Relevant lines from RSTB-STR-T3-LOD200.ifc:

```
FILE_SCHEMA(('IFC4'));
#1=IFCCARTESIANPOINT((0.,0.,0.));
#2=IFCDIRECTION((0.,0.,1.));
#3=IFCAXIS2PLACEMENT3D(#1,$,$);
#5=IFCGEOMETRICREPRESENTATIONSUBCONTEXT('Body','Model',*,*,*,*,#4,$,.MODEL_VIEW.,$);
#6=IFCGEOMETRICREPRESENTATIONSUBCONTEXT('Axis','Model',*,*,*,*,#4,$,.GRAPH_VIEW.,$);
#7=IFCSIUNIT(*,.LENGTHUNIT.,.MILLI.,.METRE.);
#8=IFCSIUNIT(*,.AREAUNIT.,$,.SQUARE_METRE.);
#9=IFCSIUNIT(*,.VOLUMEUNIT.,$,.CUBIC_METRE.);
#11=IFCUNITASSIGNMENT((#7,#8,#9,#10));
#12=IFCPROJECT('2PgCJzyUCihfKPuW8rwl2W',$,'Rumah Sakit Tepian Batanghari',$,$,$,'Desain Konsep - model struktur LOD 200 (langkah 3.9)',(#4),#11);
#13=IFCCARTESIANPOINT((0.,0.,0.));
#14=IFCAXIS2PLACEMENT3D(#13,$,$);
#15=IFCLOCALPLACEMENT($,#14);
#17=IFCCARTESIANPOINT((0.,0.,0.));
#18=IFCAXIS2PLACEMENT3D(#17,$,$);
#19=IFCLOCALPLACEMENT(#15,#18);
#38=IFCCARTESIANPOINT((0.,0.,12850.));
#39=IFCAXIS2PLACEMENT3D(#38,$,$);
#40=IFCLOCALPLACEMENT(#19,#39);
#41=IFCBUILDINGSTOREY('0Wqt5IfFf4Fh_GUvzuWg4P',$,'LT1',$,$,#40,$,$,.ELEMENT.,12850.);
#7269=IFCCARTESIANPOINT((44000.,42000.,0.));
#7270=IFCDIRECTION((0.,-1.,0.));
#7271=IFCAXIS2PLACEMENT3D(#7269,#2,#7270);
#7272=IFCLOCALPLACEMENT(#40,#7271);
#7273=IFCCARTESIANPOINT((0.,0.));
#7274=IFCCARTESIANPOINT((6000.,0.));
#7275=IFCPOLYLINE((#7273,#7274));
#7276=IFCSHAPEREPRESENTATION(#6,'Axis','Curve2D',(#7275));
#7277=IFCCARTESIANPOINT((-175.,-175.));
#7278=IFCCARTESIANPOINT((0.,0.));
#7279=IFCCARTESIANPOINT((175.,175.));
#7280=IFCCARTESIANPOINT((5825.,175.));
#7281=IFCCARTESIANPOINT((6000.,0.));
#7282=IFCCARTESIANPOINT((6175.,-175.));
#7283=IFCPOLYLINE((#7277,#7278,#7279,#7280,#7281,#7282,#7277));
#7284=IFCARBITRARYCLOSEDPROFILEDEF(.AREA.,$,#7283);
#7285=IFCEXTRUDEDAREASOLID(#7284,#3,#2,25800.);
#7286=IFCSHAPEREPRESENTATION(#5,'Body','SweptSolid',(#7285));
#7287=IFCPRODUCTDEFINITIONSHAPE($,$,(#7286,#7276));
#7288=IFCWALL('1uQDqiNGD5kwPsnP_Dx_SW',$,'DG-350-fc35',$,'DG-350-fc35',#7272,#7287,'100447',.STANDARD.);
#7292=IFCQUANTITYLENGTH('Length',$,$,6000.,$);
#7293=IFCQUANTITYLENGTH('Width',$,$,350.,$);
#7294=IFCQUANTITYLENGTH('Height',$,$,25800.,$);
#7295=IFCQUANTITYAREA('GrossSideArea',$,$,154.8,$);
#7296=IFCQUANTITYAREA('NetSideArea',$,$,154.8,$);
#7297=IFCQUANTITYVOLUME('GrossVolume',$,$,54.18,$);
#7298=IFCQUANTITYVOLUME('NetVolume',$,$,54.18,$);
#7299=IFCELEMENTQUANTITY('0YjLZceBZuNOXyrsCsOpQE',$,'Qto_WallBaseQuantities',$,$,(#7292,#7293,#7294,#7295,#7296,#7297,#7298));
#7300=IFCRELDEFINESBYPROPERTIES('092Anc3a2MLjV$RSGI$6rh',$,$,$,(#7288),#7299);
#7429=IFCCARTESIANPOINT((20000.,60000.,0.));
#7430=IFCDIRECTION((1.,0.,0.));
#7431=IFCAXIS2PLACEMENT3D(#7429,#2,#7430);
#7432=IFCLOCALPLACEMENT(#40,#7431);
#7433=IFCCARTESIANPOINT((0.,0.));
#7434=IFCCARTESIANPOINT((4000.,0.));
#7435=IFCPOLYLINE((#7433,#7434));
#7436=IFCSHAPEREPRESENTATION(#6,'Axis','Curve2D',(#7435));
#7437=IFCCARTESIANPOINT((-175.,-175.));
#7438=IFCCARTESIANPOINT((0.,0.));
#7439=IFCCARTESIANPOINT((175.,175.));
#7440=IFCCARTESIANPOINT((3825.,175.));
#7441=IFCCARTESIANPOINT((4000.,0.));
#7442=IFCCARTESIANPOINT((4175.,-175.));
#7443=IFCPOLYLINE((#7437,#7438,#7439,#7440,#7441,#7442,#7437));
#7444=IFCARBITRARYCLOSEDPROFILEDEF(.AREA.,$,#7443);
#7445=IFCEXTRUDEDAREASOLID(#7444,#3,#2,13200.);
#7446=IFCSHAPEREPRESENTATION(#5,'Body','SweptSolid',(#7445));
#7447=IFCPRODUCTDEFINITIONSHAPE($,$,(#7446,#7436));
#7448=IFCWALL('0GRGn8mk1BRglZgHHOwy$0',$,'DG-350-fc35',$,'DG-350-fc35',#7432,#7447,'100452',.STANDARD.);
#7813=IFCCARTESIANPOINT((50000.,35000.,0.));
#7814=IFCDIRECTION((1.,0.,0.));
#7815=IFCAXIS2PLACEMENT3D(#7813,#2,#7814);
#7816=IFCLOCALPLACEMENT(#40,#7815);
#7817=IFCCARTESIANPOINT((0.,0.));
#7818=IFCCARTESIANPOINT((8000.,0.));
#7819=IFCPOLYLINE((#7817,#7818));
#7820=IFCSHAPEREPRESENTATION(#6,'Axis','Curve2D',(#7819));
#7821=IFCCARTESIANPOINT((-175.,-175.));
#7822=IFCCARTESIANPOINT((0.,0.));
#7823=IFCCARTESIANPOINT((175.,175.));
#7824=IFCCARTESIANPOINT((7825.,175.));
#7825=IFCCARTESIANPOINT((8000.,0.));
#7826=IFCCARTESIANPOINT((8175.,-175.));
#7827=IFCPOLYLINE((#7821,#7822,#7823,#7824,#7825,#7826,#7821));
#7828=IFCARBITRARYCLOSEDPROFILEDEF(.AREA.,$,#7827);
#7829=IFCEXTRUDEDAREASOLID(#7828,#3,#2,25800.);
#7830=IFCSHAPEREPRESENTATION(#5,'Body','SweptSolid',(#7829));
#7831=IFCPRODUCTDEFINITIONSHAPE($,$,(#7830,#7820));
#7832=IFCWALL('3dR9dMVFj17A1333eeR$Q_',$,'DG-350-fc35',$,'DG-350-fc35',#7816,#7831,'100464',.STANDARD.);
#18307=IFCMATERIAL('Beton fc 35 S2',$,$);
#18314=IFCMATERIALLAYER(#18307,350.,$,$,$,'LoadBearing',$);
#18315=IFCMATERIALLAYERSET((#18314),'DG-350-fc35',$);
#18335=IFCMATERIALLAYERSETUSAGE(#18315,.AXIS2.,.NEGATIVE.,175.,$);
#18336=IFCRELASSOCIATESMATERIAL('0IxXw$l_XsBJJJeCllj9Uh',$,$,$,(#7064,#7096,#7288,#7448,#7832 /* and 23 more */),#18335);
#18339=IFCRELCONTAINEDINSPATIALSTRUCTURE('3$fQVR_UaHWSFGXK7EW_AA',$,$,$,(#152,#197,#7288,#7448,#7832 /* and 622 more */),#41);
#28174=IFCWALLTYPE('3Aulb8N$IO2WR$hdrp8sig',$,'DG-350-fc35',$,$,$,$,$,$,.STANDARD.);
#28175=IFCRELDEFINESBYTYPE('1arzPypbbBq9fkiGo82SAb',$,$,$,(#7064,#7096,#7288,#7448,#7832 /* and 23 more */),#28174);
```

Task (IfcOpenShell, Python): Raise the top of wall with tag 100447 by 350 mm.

```python
import ifcopenshell
import ifcopenshell.api.pset
import ifcopenshell.geom
import ifcopenshell.util.element
import ifcopenshell.util.representation
import ifcopenshell.util.shape
import ifcopenshell.util.unit

model = ifcopenshell.open("RSTB-STR-T3-LOD200.ifc")
unit_scale = ifcopenshell.util.unit.calculate_unit_scale(model)
area_scale = ifcopenshell.util.unit.calculate_unit_scale(model, "AREAUNIT")
volume_scale = ifcopenshell.util.unit.calculate_unit_scale(model, "VOLUMEUNIT")
settings = ifcopenshell.geom.settings()


def volume(element):
    """Net volume in cubic metres, openings subtracted."""
    shape = ifcopenshell.geom.create_shape(settings, element)
    return ifcopenshell.util.shape.get_volume(shape.geometry)


wall = model.by_guid("1uQDqiNGD5kwPsnP_Dx_SW")
before = volume(wall)

body = ifcopenshell.util.representation.get_representation(wall, "Model", "Body")
solid = body.Items[0]
old_height = solid.Depth
solid.Depth += 350.0
after = volume(wall)
thickness = 0.35  # wall thickness in metres

# Update the stored height, areas and volumes.
qto = model.by_id(ifcopenshell.util.element.get_pset(wall, "Qto_WallBaseQuantities", should_inherit=False)["id"])
ifcopenshell.api.pset.edit_qto(model, qto=qto, properties={
    "Height": solid.Depth,
    "GrossSideArea": ifcopenshell.util.element.get_pset(wall, "Qto_WallBaseQuantities", "GrossSideArea") * solid.Depth / old_height,
    "NetSideArea": after / thickness / area_scale,
    "GrossVolume": ifcopenshell.util.element.get_pset(wall, "Qto_WallBaseQuantities", "GrossVolume") * solid.Depth / old_height,
    "NetVolume": after / volume_scale,
})

print(f"height {old_height:g} -> {solid.Depth:g}, volume {before:.3f} -> {after:.3f} m3")

model.write("RSTB-STR-T3-LOD200_updated.ifc")
```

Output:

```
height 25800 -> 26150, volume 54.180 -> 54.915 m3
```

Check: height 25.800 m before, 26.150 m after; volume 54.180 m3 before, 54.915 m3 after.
